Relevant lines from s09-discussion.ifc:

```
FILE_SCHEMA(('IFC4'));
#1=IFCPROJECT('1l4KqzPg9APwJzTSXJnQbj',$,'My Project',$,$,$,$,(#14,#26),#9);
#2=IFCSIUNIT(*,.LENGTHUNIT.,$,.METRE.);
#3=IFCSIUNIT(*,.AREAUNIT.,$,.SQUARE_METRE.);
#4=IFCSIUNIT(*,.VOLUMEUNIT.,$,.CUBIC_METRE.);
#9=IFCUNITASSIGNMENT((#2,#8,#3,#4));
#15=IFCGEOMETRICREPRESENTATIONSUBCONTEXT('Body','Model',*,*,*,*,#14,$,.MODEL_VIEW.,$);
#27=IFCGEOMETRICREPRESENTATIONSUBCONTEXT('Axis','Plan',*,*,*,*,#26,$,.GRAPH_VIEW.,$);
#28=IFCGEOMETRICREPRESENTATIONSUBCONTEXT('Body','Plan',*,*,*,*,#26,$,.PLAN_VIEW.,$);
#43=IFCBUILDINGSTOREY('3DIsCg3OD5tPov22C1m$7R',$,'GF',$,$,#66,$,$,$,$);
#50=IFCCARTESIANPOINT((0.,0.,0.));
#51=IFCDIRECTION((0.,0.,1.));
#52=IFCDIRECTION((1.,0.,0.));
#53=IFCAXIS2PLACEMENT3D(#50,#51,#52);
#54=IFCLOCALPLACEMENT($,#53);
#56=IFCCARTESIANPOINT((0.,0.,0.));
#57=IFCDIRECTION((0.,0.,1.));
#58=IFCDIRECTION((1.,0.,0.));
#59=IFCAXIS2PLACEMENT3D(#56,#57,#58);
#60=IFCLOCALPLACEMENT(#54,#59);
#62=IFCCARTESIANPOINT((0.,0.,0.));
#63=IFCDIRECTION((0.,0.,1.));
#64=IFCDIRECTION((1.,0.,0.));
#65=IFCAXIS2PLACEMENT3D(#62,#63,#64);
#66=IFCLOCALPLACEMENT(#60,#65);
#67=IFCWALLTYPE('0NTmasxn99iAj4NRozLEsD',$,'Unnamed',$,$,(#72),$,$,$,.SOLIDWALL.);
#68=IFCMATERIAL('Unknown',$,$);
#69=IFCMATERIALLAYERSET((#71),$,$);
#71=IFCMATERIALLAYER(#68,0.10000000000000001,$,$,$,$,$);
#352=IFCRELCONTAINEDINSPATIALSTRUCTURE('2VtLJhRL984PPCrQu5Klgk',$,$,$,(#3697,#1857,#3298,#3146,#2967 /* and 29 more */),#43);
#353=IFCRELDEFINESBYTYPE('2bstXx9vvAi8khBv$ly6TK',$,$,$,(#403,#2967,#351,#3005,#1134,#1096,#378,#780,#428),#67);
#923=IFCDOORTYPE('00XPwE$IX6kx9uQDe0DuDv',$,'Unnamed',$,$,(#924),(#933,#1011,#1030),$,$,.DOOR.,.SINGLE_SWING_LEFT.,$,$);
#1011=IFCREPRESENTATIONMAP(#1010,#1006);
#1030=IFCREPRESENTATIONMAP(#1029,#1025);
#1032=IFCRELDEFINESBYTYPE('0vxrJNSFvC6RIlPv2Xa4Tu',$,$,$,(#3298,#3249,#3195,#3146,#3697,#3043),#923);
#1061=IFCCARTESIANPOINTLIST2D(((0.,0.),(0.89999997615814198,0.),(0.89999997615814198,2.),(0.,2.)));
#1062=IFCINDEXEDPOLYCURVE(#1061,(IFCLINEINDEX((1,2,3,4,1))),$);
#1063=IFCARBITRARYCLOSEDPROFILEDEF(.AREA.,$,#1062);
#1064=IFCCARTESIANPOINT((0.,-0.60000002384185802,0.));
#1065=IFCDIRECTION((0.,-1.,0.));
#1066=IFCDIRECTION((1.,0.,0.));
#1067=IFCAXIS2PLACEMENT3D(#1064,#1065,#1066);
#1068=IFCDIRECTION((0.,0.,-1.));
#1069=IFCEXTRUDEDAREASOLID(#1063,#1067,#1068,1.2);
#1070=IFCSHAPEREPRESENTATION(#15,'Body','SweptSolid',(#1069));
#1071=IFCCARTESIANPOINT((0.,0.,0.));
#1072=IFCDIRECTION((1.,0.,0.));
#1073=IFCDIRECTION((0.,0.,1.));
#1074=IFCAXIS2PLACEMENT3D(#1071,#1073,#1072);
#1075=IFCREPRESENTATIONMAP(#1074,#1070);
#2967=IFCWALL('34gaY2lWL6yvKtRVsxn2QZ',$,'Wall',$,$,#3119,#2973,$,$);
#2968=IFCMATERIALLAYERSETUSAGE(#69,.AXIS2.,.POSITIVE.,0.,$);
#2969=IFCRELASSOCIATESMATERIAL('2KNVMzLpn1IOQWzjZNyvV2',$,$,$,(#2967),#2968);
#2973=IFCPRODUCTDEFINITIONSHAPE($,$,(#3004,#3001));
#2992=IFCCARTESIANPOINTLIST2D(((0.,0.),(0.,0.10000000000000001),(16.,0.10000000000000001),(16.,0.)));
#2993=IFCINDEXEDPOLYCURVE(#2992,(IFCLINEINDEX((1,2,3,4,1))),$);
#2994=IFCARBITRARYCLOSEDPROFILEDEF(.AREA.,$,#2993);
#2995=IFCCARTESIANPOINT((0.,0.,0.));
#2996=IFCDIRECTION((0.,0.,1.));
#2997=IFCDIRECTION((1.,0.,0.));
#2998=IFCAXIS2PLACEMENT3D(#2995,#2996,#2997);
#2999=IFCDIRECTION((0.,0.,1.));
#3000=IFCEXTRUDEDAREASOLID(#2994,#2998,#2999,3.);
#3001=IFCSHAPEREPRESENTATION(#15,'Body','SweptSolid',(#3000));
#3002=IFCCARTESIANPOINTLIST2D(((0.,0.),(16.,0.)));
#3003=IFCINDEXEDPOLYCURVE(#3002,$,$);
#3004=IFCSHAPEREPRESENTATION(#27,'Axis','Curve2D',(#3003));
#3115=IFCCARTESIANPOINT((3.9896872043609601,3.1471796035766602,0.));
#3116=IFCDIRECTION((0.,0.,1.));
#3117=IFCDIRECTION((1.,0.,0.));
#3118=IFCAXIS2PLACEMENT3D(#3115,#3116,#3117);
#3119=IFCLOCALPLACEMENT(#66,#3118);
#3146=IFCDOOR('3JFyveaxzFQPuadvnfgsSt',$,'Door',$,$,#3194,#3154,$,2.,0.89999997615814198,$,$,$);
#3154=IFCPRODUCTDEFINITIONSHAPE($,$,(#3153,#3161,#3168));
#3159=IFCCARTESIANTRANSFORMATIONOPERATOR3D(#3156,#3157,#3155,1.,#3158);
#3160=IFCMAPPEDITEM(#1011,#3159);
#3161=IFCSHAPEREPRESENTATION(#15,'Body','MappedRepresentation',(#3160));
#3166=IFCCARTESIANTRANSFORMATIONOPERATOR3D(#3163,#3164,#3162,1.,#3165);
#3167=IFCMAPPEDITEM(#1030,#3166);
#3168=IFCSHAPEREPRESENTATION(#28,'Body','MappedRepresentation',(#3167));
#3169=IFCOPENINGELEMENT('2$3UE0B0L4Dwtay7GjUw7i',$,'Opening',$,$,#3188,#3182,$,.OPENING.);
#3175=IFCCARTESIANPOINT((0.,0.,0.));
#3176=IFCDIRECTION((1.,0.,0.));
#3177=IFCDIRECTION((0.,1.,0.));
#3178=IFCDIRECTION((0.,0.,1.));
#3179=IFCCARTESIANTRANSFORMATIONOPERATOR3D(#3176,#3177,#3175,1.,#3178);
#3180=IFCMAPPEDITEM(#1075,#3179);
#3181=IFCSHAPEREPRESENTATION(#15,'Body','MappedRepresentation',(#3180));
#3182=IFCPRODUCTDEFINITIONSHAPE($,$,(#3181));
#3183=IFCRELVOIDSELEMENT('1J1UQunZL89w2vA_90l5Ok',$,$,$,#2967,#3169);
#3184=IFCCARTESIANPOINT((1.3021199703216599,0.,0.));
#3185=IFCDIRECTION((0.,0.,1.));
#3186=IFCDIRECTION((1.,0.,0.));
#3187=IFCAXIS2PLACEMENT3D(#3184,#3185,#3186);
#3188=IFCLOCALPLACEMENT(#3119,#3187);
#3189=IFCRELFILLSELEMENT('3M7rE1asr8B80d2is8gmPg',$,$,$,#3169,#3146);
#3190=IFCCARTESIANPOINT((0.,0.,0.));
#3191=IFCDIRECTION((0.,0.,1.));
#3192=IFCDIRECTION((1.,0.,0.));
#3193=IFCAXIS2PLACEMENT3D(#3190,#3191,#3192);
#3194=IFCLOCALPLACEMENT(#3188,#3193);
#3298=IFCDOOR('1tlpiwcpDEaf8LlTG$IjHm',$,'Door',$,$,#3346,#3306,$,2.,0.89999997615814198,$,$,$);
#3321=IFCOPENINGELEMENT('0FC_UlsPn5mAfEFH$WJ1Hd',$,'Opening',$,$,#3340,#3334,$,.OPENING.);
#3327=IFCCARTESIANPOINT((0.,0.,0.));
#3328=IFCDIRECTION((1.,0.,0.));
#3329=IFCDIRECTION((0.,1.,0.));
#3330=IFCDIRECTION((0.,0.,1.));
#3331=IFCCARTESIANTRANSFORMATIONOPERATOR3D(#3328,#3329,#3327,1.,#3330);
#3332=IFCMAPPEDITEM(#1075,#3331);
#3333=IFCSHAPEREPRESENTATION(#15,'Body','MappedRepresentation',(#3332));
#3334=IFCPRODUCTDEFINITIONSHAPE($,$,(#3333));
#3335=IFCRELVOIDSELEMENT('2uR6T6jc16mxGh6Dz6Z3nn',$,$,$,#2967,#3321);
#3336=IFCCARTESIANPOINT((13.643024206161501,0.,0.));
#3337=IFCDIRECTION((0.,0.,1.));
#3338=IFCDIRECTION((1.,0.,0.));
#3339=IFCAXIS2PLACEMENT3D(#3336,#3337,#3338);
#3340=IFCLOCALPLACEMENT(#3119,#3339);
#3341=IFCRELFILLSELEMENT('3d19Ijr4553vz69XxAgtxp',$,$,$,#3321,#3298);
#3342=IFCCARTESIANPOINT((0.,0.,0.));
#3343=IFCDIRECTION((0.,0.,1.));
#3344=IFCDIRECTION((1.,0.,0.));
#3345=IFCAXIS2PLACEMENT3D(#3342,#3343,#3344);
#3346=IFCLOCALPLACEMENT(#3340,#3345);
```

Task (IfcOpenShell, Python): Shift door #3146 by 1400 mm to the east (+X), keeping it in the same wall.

```python
import ifcopenshell
import ifcopenshell.api.geometry
import ifcopenshell.util.placement

model = ifcopenshell.open("s09-discussion.ifc")

door = model.by_id(3146)
opening = door.FillsVoids[0].RelatingOpeningElement
wall = opening.VoidsElements[0].RelatingBuildingElement

wall_matrix = ifcopenshell.util.placement.get_local_placement(wall.ObjectPlacement)
shift = wall_matrix[:3, 0] * 1.4
before = ifcopenshell.util.placement.get_local_placement(door.ObjectPlacement)[:3, 3].copy()

# The door is placed relative to its opening, so it follows when the opening moves.
matrix = ifcopenshell.util.placement.get_local_placement(opening.ObjectPlacement)
matrix[:3, 3] += shift
ifcopenshell.api.geometry.edit_object_placement(
    model, product=opening, matrix=matrix, is_si=False, should_transform_children=True
)

after = ifcopenshell.util.placement.get_local_placement(door.ObjectPlacement)[:3, 3]
print("door moved by", (after - before).round(3) + 0.0)

model.write("s09-discussion_edited.ifc")
```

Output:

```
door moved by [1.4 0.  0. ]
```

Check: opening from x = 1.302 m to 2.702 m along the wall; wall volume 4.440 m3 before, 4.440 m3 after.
